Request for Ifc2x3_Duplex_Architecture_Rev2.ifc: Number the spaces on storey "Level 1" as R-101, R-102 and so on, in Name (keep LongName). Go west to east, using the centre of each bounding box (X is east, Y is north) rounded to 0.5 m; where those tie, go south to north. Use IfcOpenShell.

First a look at what the model holds.

```python
import ifcopenshell
import ifcopenshell.util.element
import ifcopenshell.util.placement

model = ifcopenshell.open("Ifc2x3_Duplex_Architecture_Rev2.ifc")
print(model.schema)
storey = next(s for s in model.by_type("IfcBuildingStorey") if s.Name == "Level 1")
spaces = [e for e in ifcopenshell.util.element.get_decomposition(storey) if e.is_a("IfcSpace")]
for e in sorted(spaces, key=lambda e: e.id()):
    origin = ifcopenshell.util.placement.get_local_placement(e.ObjectPlacement)[:3, 3]
    print(e.id(), e.Name, e.LongName, origin.round(2) + 0.0, sep=" | ")
```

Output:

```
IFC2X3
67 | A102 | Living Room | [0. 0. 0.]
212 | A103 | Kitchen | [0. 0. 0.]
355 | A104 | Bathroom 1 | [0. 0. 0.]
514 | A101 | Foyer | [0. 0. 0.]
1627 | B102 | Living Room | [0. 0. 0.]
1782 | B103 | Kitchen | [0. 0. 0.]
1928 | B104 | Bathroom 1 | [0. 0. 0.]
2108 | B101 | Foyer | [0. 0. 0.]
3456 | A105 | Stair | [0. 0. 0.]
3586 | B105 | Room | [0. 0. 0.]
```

```python
import ifcopenshell
import ifcopenshell.geom
import ifcopenshell.util.element
import ifcopenshell.util.shape

model = ifcopenshell.open("Ifc2x3_Duplex_Architecture_Rev2.ifc")
settings = ifcopenshell.geom.settings()
settings.set("use-world-coords", True)


def centre(element):
    shape = ifcopenshell.geom.create_shape(settings, element)
    return ifcopenshell.util.shape.get_bbox_centroid(shape.geometry)


storey = next(s for s in model.by_type("IfcBuildingStorey") if s.Name == "Level 1")
spaces = [e for e in ifcopenshell.util.element.get_decomposition(storey) if e.is_a("IfcSpace")]

# Insertion points can sit at a corner or the storey origin, so sort by the geometry (in metres).
centres = {e: centre(e) for e in spaces}
spaces.sort(key=lambda e: (round(centres[e][0] / 0.5), centres[e][1]))

for i, e in enumerate(spaces, start=1):
    number = f"R-1{i:02d}"
    e.Name = number
    print(e.id(), number)

model.write("Ifc2x3_Duplex_Architecture_Rev2-out.ifc")
```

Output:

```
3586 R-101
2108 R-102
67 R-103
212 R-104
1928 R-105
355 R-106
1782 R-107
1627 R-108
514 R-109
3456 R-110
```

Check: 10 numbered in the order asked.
